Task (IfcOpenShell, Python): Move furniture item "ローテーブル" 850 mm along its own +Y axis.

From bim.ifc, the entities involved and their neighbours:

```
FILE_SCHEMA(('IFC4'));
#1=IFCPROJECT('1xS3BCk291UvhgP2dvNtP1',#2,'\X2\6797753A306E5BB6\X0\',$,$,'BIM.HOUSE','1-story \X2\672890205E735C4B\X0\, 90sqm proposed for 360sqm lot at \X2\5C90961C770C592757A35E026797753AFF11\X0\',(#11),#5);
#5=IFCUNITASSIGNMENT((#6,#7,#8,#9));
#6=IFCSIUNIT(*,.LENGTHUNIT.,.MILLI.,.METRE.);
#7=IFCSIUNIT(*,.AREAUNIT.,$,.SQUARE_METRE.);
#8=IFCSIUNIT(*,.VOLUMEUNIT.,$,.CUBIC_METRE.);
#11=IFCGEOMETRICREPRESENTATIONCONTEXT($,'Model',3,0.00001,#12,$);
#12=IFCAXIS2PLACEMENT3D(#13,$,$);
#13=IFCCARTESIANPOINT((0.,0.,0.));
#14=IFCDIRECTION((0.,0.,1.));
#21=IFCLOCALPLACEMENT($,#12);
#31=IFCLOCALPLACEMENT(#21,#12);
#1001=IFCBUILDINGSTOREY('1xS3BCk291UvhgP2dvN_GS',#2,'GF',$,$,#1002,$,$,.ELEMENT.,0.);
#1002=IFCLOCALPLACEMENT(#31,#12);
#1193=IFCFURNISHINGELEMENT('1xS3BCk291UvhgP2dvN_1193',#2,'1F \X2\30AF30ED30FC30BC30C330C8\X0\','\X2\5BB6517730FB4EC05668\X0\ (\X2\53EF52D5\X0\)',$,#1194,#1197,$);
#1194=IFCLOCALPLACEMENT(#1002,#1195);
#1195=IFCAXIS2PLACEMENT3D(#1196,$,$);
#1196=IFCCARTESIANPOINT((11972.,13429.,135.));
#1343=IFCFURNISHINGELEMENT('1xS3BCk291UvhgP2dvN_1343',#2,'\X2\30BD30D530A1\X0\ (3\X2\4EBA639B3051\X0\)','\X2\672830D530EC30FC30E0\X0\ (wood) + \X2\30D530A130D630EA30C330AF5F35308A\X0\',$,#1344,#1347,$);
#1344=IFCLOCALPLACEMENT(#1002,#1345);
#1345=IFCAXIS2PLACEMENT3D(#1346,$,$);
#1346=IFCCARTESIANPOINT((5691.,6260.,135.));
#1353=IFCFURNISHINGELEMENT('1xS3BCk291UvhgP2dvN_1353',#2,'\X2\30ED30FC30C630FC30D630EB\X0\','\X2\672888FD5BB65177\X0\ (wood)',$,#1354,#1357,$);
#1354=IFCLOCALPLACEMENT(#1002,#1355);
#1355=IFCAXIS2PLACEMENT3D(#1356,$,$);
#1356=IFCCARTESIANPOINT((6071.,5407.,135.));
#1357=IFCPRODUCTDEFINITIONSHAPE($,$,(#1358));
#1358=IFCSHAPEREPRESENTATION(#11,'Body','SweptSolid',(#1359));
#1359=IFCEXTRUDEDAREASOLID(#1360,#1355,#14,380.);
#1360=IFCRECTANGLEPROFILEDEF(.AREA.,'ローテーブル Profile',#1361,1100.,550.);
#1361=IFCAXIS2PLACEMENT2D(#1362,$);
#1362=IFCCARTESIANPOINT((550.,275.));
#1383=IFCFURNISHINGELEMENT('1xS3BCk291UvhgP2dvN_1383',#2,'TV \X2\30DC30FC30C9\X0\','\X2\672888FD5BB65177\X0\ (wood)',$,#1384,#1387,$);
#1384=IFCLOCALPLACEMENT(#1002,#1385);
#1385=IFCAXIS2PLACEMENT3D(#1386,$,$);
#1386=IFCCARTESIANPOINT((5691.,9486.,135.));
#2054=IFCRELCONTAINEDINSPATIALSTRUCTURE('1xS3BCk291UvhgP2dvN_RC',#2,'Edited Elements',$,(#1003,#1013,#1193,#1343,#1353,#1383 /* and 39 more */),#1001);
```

```python
import ifcopenshell
import ifcopenshell.api.geometry
import ifcopenshell.util.placement
import ifcopenshell.util.unit

model = ifcopenshell.open("bim.ifc")
unit_scale = ifcopenshell.util.unit.calculate_unit_scale(model)

item = model.by_guid("1xS3BCk291UvhgP2dvN_1353")
matrix = ifcopenshell.util.placement.get_local_placement(item.ObjectPlacement)
matrix[:3, 3] += matrix[:3, 1] * 0.85 / unit_scale
ifcopenshell.api.geometry.edit_object_placement(model, product=item, matrix=matrix, is_si=False)

print(ifcopenshell.util.placement.get_local_placement(item.ObjectPlacement).round(3) + 0.0)

model.write("bim_updated.ifc")
```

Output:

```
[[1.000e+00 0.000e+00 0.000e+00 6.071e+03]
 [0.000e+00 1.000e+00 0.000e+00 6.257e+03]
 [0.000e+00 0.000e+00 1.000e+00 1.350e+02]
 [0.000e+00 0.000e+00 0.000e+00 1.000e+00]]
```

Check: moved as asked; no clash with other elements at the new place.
